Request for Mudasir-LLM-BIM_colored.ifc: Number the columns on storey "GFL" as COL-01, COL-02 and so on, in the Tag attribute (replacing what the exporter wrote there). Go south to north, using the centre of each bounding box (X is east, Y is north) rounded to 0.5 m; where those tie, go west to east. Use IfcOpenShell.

First a look at what the model holds.

```python
import ifcopenshell
import ifcopenshell.util.element
import ifcopenshell.util.placement

model = ifcopenshell.open("Mudasir-LLM-BIM_colored.ifc")
print(model.schema)
storey = next(s for s in model.by_type("IfcBuildingStorey") if s.Name == "GFL")
columns = [e for e in ifcopenshell.util.element.get_decomposition(storey) if e.is_a("IfcColumn")]
for e in sorted(columns, key=lambda e: e.id()):
    origin = ifcopenshell.util.placement.get_local_placement(e.ObjectPlacement)[:3, 3]
    print(e.id(), e.Tag, e.Name, origin.round(2) + 0.0, sep=" | ")
```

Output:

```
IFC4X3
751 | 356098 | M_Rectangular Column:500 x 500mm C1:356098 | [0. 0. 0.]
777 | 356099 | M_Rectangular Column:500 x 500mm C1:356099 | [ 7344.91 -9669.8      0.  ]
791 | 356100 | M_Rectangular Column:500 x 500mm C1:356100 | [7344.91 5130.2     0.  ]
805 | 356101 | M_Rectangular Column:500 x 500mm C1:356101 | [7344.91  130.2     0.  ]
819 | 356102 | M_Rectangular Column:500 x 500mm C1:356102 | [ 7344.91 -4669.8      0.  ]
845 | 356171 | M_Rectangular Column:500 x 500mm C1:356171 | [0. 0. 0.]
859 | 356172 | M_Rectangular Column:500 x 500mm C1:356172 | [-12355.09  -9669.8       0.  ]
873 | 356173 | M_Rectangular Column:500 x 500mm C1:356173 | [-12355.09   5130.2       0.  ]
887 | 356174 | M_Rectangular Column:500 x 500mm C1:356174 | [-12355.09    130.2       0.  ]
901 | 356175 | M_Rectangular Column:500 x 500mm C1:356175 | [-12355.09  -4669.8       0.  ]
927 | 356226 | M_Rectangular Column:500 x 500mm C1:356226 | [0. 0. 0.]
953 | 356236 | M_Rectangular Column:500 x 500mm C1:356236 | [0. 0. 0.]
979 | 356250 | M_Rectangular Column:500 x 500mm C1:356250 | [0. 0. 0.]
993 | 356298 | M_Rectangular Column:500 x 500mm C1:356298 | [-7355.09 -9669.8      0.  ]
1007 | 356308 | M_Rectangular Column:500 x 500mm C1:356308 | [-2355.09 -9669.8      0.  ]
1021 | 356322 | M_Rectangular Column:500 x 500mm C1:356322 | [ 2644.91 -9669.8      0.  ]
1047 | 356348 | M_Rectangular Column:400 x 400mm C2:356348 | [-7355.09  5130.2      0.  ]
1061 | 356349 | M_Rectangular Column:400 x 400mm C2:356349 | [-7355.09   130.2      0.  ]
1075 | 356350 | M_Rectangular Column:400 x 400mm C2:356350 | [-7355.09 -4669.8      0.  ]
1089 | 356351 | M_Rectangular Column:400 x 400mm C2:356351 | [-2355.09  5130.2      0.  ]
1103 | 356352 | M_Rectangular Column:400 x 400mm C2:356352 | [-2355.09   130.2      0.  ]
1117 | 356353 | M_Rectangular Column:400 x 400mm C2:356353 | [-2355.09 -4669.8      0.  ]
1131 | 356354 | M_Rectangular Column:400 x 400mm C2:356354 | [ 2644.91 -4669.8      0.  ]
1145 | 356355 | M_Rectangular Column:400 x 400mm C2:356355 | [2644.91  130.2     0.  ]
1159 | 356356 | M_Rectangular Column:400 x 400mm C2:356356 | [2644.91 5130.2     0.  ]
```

```python
import ifcopenshell
import ifcopenshell.geom
import ifcopenshell.util.element
import ifcopenshell.util.shape

model = ifcopenshell.open("Mudasir-LLM-BIM_colored.ifc")
settings = ifcopenshell.geom.settings()
settings.set("use-world-coords", True)


def centre(element):
    shape = ifcopenshell.geom.create_shape(settings, element)
    return ifcopenshell.util.shape.get_bbox_centroid(shape.geometry)


storey = next(s for s in model.by_type("IfcBuildingStorey") if s.Name == "GFL")
columns = [e for e in ifcopenshell.util.element.get_decomposition(storey) if e.is_a("IfcColumn")]

# Insertion points can sit at a corner or the storey origin, so sort by the geometry (in metres).
centres = {e: centre(e) for e in columns}
columns.sort(key=lambda e: (round(centres[e][1] / 0.5), centres[e][0]))

for i, e in enumerate(columns, start=1):
    number = f"COL-{i:02d}"
    e.Tag = number
    print(e.id(), number)

model.write("Mudasir-LLM-BIM_colored_v2.ifc")
```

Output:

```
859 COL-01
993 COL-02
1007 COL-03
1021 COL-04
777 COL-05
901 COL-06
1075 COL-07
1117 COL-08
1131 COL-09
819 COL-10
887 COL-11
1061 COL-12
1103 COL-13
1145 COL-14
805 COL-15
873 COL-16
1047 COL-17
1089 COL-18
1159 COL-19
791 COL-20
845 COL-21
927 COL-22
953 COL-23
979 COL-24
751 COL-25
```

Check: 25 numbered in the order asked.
